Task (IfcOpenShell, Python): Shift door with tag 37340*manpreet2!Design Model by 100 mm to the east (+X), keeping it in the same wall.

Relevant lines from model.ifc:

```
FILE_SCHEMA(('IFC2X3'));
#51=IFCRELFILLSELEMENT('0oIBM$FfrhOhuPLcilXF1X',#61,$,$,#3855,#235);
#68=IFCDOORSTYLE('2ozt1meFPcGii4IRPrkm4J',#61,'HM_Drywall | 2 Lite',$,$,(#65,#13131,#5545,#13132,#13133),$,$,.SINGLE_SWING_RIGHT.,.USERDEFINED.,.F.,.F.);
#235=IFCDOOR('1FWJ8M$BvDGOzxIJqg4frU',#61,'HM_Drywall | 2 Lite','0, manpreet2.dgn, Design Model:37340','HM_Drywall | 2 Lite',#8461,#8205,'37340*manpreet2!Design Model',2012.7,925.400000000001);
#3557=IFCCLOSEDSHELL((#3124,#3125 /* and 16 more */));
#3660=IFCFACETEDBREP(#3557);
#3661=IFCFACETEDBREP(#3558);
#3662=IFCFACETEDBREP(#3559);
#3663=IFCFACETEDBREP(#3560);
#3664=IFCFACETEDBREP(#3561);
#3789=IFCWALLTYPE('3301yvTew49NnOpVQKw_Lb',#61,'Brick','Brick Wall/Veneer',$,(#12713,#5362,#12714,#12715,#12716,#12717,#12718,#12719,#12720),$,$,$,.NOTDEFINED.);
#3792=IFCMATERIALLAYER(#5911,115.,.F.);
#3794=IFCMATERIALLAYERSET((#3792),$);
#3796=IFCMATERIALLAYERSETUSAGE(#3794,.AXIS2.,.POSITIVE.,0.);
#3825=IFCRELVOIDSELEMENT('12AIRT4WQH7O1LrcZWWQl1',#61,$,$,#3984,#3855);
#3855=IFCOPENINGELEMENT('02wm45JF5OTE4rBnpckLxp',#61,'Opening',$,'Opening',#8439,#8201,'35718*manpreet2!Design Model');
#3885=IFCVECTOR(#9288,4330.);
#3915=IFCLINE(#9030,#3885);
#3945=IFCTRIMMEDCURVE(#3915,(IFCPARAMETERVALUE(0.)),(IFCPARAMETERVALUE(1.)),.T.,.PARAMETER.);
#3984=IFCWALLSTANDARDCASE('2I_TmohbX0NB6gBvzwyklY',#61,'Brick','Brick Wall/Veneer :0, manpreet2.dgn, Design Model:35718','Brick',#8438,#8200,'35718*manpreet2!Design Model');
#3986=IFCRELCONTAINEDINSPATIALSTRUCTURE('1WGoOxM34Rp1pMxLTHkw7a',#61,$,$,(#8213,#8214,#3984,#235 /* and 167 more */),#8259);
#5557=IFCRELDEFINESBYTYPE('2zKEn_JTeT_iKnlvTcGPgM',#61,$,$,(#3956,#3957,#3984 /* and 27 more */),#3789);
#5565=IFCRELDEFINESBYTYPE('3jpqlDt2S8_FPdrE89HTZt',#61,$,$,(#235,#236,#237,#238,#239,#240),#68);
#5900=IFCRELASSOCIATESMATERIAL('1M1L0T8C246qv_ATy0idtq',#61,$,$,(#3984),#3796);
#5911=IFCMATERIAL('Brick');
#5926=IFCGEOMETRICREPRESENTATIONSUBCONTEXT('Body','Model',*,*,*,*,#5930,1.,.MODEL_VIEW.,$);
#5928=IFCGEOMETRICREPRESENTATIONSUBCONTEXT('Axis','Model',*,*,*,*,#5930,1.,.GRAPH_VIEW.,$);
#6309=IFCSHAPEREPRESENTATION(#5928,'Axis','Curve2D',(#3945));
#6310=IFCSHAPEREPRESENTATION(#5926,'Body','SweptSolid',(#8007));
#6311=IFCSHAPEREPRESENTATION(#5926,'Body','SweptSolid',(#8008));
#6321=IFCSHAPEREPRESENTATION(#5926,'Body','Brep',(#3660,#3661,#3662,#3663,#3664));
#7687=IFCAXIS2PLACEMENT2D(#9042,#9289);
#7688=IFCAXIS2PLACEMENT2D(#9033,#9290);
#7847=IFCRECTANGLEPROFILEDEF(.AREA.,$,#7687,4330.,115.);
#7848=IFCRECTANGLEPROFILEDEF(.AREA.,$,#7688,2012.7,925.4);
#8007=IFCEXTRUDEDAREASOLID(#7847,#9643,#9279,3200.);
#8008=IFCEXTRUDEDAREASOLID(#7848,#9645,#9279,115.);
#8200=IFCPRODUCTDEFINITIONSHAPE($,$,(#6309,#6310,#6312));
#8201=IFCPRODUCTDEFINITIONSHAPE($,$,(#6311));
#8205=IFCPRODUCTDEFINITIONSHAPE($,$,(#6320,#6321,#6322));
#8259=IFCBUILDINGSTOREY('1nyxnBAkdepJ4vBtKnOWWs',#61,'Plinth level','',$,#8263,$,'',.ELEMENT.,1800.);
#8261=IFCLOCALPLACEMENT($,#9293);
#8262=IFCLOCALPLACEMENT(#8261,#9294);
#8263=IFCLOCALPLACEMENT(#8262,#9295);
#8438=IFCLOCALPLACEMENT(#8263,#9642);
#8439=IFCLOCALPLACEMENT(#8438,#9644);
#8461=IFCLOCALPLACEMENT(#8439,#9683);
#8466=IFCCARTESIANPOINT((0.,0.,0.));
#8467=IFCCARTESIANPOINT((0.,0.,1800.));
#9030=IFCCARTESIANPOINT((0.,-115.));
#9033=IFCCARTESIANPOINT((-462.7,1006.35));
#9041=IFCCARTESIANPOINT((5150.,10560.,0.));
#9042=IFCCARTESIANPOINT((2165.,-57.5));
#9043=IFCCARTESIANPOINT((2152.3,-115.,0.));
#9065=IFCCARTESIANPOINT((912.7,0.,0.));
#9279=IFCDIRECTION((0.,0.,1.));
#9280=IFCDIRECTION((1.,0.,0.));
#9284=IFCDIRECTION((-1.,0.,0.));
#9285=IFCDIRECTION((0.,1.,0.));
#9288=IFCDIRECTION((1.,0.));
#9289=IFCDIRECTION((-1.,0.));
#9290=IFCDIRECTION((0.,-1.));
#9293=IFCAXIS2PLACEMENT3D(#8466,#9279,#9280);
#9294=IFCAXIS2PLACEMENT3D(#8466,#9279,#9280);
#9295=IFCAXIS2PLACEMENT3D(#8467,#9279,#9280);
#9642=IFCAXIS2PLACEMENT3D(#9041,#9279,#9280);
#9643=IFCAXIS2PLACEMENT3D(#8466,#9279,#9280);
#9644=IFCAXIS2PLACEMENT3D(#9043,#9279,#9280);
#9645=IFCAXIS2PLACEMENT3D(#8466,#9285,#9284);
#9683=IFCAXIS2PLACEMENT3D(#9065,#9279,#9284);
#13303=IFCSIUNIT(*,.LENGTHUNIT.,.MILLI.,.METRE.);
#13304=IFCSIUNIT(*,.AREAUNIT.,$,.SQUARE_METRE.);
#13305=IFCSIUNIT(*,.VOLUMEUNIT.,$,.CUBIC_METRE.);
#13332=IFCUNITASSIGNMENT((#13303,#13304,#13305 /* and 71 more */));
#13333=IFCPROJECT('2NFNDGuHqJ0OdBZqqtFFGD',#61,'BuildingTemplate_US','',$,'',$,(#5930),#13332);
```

```python
import ifcopenshell
import ifcopenshell.api.geometry
import ifcopenshell.util.placement
import ifcopenshell.util.unit

model = ifcopenshell.open("model.ifc")
unit_scale = ifcopenshell.util.unit.calculate_unit_scale(model)

door = model.by_guid("1FWJ8M$BvDGOzxIJqg4frU")
opening = door.FillsVoids[0].RelatingOpeningElement
wall = opening.VoidsElements[0].RelatingBuildingElement

wall_matrix = ifcopenshell.util.placement.get_local_placement(wall.ObjectPlacement)
shift = wall_matrix[:3, 0] * 0.1 / unit_scale
before = ifcopenshell.util.placement.get_local_placement(door.ObjectPlacement)[:3, 3].copy()

# The door is placed relative to its opening, so it follows when the opening moves.
matrix = ifcopenshell.util.placement.get_local_placement(opening.ObjectPlacement)
matrix[:3, 3] += shift
ifcopenshell.api.geometry.edit_object_placement(
    model, product=opening, matrix=matrix, is_si=False, should_transform_children=True
)

after = ifcopenshell.util.placement.get_local_placement(door.ObjectPlacement)[:3, 3]
print("door moved by", (after - before).round(3) + 0.0)

model.write("model_updated.ifc")
```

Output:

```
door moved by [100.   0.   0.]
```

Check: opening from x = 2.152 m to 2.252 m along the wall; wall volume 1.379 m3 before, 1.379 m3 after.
